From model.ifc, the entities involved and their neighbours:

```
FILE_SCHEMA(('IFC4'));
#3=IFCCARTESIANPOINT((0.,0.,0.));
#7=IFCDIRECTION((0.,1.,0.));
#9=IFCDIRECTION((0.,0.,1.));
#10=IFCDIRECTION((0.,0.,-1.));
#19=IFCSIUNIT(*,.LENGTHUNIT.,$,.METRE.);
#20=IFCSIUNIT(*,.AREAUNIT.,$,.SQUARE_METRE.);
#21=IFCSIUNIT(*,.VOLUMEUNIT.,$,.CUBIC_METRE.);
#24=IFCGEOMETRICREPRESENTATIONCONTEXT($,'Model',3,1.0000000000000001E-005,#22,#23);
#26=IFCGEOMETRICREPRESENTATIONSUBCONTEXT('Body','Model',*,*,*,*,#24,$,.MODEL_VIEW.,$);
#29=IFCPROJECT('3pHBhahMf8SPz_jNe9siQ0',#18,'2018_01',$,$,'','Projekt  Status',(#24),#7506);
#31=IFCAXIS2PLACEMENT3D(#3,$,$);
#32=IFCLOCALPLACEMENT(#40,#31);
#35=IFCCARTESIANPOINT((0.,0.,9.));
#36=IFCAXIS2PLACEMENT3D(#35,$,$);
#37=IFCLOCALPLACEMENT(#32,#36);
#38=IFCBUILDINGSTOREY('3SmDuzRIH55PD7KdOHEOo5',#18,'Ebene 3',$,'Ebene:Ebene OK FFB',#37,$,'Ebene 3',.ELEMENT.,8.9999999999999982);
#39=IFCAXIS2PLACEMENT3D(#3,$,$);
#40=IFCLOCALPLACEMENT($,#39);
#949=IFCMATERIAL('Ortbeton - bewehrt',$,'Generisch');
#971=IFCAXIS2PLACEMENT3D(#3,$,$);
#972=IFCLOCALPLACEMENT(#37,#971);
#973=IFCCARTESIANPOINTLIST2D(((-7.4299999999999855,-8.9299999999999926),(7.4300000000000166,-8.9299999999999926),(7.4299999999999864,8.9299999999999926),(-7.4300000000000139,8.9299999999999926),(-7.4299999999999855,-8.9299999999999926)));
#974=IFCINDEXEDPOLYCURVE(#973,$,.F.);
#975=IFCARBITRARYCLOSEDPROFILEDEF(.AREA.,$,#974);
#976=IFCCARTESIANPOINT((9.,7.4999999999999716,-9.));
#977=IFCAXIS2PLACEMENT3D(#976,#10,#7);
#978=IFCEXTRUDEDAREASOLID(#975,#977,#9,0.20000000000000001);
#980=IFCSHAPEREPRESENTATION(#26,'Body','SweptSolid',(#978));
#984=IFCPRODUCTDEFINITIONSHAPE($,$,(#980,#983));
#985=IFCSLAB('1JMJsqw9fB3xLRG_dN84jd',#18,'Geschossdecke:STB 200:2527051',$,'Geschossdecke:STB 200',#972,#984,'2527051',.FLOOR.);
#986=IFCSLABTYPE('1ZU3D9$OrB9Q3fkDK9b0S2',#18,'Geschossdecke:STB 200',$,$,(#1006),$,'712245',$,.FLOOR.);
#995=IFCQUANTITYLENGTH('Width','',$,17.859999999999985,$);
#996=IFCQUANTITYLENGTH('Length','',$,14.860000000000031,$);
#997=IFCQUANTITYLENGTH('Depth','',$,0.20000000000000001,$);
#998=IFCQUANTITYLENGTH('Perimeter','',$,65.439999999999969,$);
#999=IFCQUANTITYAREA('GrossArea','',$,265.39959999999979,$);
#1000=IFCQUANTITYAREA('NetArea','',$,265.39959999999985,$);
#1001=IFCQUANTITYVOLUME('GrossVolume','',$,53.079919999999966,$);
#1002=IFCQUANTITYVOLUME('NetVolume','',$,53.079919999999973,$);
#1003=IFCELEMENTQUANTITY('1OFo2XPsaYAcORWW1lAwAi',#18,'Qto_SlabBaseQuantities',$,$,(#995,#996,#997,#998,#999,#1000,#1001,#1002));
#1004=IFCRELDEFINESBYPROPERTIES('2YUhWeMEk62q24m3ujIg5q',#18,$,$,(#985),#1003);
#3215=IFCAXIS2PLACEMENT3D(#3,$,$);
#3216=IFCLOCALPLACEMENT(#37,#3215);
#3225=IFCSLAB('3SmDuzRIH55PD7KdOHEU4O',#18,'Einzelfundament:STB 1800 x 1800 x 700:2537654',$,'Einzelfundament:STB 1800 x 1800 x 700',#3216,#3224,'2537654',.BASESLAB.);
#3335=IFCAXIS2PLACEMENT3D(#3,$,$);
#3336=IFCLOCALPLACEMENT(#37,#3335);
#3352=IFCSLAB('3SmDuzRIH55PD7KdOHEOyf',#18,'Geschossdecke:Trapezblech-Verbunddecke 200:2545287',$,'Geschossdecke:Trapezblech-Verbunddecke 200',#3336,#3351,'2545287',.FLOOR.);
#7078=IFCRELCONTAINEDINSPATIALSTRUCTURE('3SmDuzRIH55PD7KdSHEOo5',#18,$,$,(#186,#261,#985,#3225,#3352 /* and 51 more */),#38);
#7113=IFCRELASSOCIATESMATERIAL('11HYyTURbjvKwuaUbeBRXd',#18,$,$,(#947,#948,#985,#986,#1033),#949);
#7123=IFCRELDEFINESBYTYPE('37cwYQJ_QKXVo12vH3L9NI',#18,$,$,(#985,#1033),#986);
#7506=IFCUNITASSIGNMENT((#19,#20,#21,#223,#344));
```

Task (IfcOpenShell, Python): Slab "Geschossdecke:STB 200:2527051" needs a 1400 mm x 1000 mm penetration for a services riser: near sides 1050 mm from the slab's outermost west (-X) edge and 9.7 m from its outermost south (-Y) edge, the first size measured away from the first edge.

```python
import numpy as np
import ifcopenshell
import ifcopenshell.api.feature
import ifcopenshell.api.geometry
import ifcopenshell.api.pset
import ifcopenshell.api.root
import ifcopenshell.geom
import ifcopenshell.util.element
import ifcopenshell.util.placement
import ifcopenshell.util.representation
import ifcopenshell.util.shape
import ifcopenshell.util.unit

model = ifcopenshell.open("model.ifc")
unit_scale = ifcopenshell.util.unit.calculate_unit_scale(model)
area_scale = ifcopenshell.util.unit.calculate_unit_scale(model, "AREAUNIT")
volume_scale = ifcopenshell.util.unit.calculate_unit_scale(model, "VOLUMEUNIT")
settings = ifcopenshell.geom.settings()


def volume(element):
    """Net volume in cubic metres, openings subtracted."""
    shape = ifcopenshell.geom.create_shape(settings, element)
    return ifcopenshell.util.shape.get_volume(shape.geometry)


slab = model.by_guid("1JMJsqw9fB3xLRG_dN84jd")
before = volume(slab)

# Extent in the slab's own axes, in metres. The edges named are its -X and -Y sides.
slab_shape = ifcopenshell.geom.create_shape(settings, slab)
vertices = ifcopenshell.util.shape.get_vertices(slab_shape.geometry)
x_min, y_min, bottom = vertices.min(axis=0)
top = vertices[:, 2].max()

opening = ifcopenshell.api.root.create_entity(model, ifc_class="IfcOpeningElement", name="Services riser opening", predefined_type="OPENING")
context = ifcopenshell.util.representation.get_context(model, "Model", "Body", "MODEL_VIEW")
width, depth = 1.4, 1
outline = [(0.0, 0.0), (width, 0.0), (width, depth), (0.0, depth), (0.0, 0.0)]
# Overshoot both faces by 50 mm so the cut is clean.
shape = ifcopenshell.api.geometry.add_slab_representation(
    model, context=context, depth=top - bottom + 0.1, polyline=outline
)
ifcopenshell.api.geometry.assign_representation(model, product=opening, representation=shape)

matrix = ifcopenshell.util.placement.get_local_placement(slab.ObjectPlacement)
matrix[:, 3] = matrix @ np.append(np.array([x_min + 1.05, y_min + 9.7, bottom - 0.05]) / unit_scale, 1.0)
ifcopenshell.api.geometry.edit_object_placement(model, product=opening, matrix=matrix, is_si=False)
ifcopenshell.api.feature.add_feature(model, feature=opening, element=slab)

after = volume(slab)

# Update the slab's stored quantities.
qto = model.by_id(ifcopenshell.util.element.get_pset(slab, "Qto_SlabBaseQuantities", should_inherit=False)["id"])
ifcopenshell.api.pset.edit_qto(model, qto=qto, properties={
    "NetArea": after / (top - bottom) / area_scale,
    "NetVolume": after / volume_scale,
})

print(f"slab volume {before:.3f} -> {after:.3f} m3")

model.write("model_rev.ifc")
```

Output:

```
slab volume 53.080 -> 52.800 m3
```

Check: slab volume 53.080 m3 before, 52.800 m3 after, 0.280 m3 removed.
